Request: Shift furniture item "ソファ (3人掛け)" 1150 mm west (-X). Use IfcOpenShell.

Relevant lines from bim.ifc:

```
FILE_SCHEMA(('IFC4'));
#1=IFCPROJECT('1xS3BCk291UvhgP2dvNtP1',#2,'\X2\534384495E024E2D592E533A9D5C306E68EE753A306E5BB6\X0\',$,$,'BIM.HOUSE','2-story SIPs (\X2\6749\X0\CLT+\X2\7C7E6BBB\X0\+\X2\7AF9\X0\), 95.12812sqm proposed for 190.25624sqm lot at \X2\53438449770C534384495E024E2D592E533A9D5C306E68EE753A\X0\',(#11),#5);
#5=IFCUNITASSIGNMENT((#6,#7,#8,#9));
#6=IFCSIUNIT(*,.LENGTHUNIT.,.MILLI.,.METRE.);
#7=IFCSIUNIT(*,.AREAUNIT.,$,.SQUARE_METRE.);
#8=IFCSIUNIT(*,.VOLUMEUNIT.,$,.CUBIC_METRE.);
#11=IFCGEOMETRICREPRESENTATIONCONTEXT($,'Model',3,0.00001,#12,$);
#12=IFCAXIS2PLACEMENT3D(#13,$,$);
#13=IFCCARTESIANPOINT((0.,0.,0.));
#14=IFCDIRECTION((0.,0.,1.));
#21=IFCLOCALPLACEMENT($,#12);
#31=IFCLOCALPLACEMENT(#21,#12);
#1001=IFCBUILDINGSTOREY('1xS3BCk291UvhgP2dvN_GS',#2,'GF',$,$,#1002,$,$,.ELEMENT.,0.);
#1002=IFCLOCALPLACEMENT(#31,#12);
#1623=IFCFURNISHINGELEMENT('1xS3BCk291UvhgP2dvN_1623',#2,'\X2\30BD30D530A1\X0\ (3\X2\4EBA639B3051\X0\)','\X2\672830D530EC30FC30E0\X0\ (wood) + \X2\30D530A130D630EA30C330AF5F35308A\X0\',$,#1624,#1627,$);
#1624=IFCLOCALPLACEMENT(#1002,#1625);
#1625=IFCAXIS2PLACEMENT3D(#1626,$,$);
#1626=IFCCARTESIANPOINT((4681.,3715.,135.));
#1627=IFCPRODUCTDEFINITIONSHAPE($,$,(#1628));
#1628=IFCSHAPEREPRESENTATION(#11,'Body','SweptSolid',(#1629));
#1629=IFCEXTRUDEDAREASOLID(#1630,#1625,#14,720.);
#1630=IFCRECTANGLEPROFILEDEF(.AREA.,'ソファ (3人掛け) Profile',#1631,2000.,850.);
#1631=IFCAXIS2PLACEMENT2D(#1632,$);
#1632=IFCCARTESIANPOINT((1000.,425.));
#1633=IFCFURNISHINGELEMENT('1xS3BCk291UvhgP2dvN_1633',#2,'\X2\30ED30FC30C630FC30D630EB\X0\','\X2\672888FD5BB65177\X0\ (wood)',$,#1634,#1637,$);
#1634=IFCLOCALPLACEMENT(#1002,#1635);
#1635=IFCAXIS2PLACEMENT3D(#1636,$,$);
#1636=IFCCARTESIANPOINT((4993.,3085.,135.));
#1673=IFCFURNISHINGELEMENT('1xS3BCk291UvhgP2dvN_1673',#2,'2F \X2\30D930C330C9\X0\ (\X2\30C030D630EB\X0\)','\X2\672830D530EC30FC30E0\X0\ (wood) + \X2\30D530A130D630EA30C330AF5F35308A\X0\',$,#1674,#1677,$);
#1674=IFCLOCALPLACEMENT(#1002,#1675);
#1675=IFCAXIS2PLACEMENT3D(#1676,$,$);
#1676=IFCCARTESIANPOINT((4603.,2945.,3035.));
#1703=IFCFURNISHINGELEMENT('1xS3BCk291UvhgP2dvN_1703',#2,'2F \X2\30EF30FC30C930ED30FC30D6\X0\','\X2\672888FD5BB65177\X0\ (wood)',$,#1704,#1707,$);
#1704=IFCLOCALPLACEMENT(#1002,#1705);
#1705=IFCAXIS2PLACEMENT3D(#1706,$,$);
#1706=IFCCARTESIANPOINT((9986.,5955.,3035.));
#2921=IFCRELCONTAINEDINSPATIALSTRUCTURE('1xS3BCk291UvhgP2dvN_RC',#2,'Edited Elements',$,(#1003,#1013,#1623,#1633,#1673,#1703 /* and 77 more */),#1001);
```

```python
import ifcopenshell
import ifcopenshell.api.geometry
import ifcopenshell.util.placement
import ifcopenshell.util.unit

model = ifcopenshell.open("bim.ifc")
unit_scale = ifcopenshell.util.unit.calculate_unit_scale(model)

item = model.by_guid("1xS3BCk291UvhgP2dvN_1623")
matrix = ifcopenshell.util.placement.get_local_placement(item.ObjectPlacement)
matrix[0, 3] -= 1.15 / unit_scale
ifcopenshell.api.geometry.edit_object_placement(model, product=item, matrix=matrix, is_si=False)

print(ifcopenshell.util.placement.get_local_placement(item.ObjectPlacement).round(3) + 0.0)

model.write("bim_updated.ifc")
```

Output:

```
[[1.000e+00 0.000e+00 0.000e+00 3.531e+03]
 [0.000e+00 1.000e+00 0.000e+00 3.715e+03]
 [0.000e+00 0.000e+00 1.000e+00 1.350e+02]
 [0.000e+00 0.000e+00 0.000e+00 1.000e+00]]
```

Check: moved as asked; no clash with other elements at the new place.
